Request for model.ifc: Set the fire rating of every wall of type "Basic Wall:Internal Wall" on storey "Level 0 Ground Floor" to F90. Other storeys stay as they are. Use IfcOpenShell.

First a look at what the model holds.

```python
import ifcopenshell
import ifcopenshell.util.element

model = ifcopenshell.open("model.ifc")
print(model.schema)
storey = next(s for s in model.by_type("IfcBuildingStorey") if s.Name == "Level 0 Ground Floor")
walls = [e for e in ifcopenshell.util.element.get_decomposition(storey) if e.is_a("IfcWall")]
seen = {}
for e in walls:
    element_type = ifcopenshell.util.element.get_type(e)
    key = (element_type.Name if element_type != e and element_type else None, ifcopenshell.util.element.get_pset(e, "Pset_WallCommon", "FireRating"))
    seen[key] = seen.get(key, 0) + 1
for (name, value), count in sorted(seen.items(), key=str):
    print(count, "x", name, "|", value)
```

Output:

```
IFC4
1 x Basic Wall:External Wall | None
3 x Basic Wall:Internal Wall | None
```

```python
import ifcopenshell
import ifcopenshell.api.pset
import ifcopenshell.util.element

model = ifcopenshell.open("model.ifc")

storey = next(s for s in model.by_type("IfcBuildingStorey") if s.Name == "Level 0 Ground Floor")
walls = [e for e in ifcopenshell.util.element.get_decomposition(storey) if e.is_a("IfcWall")]

count = 0
for e in walls:
    element_type = ifcopenshell.util.element.get_type(e)
    if element_type in (None, e) or element_type.Name != "Basic Wall:Internal Wall":
        continue
    # add_pset returns the element's existing set when there is one.
    pset = ifcopenshell.api.pset.add_pset(model, product=e, name="Pset_WallCommon")
    ifcopenshell.api.pset.edit_pset(model, pset=pset, properties={"FireRating": "F90"})
    count += 1

print(count, "walls updated")

model.write("model-out.ifc")
```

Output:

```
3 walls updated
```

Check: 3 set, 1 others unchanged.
